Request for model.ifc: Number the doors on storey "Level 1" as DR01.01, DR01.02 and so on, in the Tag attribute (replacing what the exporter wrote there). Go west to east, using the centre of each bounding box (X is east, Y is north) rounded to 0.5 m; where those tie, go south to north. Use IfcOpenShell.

First a look at what the model holds.

```python
import ifcopenshell
import ifcopenshell.util.element
import ifcopenshell.util.placement

model = ifcopenshell.open("model.ifc")
print(model.schema)
storey = next(s for s in model.by_type("IfcBuildingStorey") if s.Name == "Level 1")
doors = [e for e in ifcopenshell.util.element.get_decomposition(storey) if e.is_a("IfcDoor")]
for e in sorted(doors, key=lambda e: e.id()):
    origin = ifcopenshell.util.placement.get_local_placement(e.ObjectPlacement)[:3, 3]
    print(e.id(), e.Tag, e.Name, origin.round(2) + 0.0, sep=" | ")
```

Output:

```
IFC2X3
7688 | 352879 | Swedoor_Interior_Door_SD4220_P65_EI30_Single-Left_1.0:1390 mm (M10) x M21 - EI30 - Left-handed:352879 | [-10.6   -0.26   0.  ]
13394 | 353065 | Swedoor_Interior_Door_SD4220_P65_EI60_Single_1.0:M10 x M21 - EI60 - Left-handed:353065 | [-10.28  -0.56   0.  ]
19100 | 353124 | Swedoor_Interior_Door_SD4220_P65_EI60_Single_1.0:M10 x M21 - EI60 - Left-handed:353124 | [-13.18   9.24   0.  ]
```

```python
import ifcopenshell
import ifcopenshell.geom
import ifcopenshell.util.element
import ifcopenshell.util.shape

model = ifcopenshell.open("model.ifc")
settings = ifcopenshell.geom.settings()
settings.set("use-world-coords", True)


def centre(element):
    shape = ifcopenshell.geom.create_shape(settings, element)
    return ifcopenshell.util.shape.get_bbox_centroid(shape.geometry)


storey = next(s for s in model.by_type("IfcBuildingStorey") if s.Name == "Level 1")
doors = [e for e in ifcopenshell.util.element.get_decomposition(storey) if e.is_a("IfcDoor")]

# Insertion points can sit at a corner or the storey origin, so sort by the geometry (in metres).
centres = {e: centre(e) for e in doors}
doors.sort(key=lambda e: (round(centres[e][0] / 0.5), centres[e][1]))

for i, e in enumerate(doors, start=1):
    number = f"DR01.{i:02d}"
    e.Tag = number
    print(e.id(), number)

model.write("model_v2.ifc")
```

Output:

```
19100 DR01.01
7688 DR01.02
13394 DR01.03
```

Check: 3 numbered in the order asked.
